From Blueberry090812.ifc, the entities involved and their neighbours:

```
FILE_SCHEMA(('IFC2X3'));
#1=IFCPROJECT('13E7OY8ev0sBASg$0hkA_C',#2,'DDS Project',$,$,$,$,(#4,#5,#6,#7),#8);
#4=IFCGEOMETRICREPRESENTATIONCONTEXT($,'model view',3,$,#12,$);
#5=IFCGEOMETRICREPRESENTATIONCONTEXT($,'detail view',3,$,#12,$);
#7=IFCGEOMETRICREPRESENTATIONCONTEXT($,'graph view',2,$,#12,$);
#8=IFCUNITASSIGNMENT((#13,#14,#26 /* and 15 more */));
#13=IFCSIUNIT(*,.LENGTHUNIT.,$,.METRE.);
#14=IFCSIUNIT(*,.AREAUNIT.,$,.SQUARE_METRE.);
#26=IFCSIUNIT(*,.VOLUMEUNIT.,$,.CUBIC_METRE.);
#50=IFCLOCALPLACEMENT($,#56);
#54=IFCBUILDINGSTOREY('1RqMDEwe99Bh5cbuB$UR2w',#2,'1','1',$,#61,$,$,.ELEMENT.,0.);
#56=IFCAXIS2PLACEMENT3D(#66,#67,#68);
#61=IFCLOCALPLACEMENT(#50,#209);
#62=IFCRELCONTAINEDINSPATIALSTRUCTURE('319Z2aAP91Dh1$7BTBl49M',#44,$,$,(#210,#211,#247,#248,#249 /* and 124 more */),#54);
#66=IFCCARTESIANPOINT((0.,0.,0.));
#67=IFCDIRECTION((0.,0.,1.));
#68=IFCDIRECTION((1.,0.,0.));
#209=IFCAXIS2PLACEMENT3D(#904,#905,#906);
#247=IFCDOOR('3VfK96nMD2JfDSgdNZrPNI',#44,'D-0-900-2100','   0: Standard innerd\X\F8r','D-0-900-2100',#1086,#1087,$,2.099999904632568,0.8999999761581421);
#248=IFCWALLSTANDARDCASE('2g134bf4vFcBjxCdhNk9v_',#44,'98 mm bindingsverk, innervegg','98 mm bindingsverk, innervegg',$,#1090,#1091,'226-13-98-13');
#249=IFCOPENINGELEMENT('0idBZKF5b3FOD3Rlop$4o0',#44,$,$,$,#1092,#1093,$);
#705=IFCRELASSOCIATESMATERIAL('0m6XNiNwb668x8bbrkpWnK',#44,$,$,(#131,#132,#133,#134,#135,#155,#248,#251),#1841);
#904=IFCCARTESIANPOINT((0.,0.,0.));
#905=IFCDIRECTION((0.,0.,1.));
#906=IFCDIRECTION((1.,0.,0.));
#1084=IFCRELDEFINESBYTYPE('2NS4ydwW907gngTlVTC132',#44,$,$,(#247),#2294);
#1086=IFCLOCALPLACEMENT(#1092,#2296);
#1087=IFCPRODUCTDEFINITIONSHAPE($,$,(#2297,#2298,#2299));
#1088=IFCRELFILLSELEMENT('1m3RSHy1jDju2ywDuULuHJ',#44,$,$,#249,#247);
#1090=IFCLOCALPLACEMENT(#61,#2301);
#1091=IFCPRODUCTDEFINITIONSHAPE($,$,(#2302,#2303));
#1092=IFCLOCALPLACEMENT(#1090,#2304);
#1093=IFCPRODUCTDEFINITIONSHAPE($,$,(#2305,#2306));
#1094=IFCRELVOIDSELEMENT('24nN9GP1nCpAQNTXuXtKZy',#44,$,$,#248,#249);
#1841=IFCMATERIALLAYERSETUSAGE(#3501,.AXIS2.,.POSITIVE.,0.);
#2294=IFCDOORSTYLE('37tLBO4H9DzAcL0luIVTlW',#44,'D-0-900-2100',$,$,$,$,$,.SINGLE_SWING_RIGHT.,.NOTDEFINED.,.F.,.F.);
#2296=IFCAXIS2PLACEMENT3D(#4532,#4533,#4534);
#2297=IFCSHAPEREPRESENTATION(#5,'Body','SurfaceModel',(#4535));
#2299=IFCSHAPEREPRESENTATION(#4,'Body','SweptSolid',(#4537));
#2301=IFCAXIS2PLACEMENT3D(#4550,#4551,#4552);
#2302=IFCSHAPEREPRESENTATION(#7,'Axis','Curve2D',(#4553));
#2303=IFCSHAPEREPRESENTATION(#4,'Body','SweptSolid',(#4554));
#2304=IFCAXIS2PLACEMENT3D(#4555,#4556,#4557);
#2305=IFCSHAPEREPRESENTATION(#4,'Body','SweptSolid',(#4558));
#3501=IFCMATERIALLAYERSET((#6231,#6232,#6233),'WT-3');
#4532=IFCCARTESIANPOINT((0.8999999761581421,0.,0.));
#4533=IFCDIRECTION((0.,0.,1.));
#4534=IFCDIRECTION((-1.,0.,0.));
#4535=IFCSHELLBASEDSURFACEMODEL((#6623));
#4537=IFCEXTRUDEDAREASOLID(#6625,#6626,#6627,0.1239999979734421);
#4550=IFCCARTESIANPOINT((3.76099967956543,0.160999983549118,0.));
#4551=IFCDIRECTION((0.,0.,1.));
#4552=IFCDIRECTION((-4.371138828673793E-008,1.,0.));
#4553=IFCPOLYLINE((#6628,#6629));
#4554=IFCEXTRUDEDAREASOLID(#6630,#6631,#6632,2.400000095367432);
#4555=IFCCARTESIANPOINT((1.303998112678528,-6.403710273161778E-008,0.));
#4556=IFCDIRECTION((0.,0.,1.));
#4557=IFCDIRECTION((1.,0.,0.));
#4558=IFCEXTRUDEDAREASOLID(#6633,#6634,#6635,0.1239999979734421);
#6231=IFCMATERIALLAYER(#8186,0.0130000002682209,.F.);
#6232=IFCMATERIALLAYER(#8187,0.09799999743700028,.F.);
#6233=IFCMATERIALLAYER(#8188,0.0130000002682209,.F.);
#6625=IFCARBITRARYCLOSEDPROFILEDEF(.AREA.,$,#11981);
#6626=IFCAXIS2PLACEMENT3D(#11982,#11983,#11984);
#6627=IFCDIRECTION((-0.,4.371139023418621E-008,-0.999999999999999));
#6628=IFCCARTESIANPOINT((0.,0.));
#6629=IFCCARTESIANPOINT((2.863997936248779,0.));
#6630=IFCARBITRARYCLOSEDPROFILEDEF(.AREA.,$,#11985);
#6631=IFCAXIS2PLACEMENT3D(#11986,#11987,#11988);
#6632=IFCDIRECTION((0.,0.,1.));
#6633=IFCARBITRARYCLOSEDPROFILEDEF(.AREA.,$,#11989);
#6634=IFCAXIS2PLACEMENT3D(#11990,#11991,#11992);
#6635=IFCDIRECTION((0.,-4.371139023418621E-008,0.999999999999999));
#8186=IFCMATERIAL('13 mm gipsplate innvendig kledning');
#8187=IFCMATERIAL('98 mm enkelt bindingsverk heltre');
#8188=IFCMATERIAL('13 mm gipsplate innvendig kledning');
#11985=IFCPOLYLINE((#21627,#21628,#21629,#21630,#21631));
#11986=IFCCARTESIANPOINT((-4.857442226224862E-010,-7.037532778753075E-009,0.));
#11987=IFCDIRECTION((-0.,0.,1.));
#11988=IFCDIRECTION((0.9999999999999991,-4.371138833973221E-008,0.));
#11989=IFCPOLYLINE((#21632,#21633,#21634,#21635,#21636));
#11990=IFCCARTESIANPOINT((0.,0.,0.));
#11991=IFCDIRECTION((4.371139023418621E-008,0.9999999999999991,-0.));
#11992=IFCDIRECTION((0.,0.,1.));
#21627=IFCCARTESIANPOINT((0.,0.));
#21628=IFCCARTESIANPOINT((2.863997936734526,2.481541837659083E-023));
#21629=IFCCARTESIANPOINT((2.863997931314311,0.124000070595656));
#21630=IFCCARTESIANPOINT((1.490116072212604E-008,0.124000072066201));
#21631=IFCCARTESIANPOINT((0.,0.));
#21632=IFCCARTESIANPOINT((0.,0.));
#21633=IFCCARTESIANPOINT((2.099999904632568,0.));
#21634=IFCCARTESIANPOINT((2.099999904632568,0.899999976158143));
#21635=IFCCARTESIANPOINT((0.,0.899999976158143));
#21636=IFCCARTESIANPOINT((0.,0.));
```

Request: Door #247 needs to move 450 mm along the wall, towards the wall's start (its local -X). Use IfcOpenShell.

```python
import ifcopenshell
import ifcopenshell.api.geometry
import ifcopenshell.util.placement
import ifcopenshell.util.unit

model = ifcopenshell.open("Blueberry090812.ifc")
unit_scale = ifcopenshell.util.unit.calculate_unit_scale(model)

door = model.by_id(247)
opening = door.FillsVoids[0].RelatingOpeningElement
wall = opening.VoidsElements[0].RelatingBuildingElement

wall_matrix = ifcopenshell.util.placement.get_local_placement(wall.ObjectPlacement)
shift = wall_matrix[:3, 0] * -0.45 / unit_scale
before = ifcopenshell.util.placement.get_local_placement(door.ObjectPlacement)[:3, 3].copy()

# The door is placed relative to its opening, so it follows when the opening moves.
matrix = ifcopenshell.util.placement.get_local_placement(opening.ObjectPlacement)
matrix[:3, 3] += shift
ifcopenshell.api.geometry.edit_object_placement(
    model, product=opening, matrix=matrix, is_si=False, should_transform_children=True
)

after = ifcopenshell.util.placement.get_local_placement(door.ObjectPlacement)[:3, 3]
print("door moved by", (after - before).round(3) + 0.0)

model.write("Blueberry090812_edited.ifc")
```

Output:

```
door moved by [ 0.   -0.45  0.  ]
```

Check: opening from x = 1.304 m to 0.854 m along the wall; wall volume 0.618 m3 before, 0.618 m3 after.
